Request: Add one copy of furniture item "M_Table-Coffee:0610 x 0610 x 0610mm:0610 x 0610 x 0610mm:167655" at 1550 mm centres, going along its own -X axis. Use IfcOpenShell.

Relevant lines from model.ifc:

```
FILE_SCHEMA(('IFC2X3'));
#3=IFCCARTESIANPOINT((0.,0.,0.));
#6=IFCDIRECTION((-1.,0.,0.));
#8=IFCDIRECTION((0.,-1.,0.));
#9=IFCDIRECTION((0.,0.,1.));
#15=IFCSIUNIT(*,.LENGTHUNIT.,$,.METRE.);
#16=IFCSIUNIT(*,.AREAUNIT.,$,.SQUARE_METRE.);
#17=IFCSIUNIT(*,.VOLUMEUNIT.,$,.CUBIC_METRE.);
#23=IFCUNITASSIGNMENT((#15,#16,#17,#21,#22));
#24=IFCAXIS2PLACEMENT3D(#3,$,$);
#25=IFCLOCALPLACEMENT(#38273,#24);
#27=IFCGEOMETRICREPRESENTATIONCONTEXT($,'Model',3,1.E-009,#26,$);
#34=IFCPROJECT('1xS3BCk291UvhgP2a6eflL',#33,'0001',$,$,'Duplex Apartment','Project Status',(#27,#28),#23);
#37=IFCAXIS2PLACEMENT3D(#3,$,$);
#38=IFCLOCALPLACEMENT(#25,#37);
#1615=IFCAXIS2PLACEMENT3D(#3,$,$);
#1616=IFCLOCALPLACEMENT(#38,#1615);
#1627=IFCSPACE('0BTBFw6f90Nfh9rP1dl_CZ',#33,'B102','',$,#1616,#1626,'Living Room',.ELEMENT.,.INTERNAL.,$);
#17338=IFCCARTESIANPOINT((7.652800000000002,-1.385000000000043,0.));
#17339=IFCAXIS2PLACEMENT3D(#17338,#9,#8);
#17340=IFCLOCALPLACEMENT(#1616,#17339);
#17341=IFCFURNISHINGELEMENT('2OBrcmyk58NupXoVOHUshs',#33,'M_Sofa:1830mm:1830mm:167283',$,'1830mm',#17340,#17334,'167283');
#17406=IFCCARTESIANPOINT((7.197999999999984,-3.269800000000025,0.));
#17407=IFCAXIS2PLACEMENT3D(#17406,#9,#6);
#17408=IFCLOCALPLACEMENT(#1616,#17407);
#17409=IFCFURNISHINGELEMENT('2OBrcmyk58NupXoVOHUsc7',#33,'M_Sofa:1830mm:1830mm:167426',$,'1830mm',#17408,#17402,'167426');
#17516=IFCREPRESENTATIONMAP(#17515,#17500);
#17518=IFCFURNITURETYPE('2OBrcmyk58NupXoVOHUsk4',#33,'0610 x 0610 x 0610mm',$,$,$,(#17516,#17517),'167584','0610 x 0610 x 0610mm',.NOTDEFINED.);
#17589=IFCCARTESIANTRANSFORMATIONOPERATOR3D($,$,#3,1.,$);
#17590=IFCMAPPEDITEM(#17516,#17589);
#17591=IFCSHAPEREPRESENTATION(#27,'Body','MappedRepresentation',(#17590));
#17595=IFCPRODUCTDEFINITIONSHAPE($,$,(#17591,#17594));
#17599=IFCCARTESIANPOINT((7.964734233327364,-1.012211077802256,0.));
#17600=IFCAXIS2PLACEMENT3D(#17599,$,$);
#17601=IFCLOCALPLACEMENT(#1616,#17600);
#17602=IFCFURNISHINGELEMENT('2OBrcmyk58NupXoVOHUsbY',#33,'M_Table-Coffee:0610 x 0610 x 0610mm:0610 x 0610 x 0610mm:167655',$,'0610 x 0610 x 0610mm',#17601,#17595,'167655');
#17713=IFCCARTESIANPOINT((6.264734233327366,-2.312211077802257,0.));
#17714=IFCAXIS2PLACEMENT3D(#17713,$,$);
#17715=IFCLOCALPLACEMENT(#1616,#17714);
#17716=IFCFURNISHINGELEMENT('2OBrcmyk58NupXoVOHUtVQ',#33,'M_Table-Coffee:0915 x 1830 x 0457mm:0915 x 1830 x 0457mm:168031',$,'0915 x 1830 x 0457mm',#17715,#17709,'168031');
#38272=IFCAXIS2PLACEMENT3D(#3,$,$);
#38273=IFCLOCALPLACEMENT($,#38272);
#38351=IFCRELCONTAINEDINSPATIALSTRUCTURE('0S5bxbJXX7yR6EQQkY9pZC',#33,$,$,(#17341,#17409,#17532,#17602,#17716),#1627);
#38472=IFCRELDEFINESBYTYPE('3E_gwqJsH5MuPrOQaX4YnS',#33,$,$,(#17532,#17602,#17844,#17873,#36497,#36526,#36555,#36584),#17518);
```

```python
import ifcopenshell
import ifcopenshell.api.geometry
import ifcopenshell.api.root
import ifcopenshell.util.element
import ifcopenshell.util.placement
import ifcopenshell.util.unit

model = ifcopenshell.open("model.ifc")
unit_scale = ifcopenshell.util.unit.calculate_unit_scale(model)


def reuse_history(source, copy):
    """copy_class also copies each property set's owner history, people and application; keep the originals."""
    for rel in copy.IsDefinedBy:
        if rel.is_a("IfcRelDefinesByProperties") and (history := rel.RelatingPropertyDefinition.OwnerHistory):
            rel.RelatingPropertyDefinition.OwnerHistory = source.OwnerHistory
            ifcopenshell.util.element.remove_deep2(model, history)


source = model.by_id(17602)
base = ifcopenshell.util.placement.get_local_placement(source.ObjectPlacement)
step = -base[:3, 0] * 1.55 / unit_scale

for i in range(1, 2):
    copy = ifcopenshell.api.root.copy_class(model, product=source)
    copy.Representation = ifcopenshell.util.element.copy_deep(
        model, source.Representation, exclude=["IfcGeometricRepresentationContext", "IfcRepresentationMap"]
    )
    copy.Name = "M_Table-Coffee:0610 x 0610 x 0610mm:0610 x 0610 x 0610mm"
    copy.Tag = None
    reuse_history(source, copy)
    matrix = base.copy()
    matrix[:3, 3] += i * step
    print("added at", matrix[:3, 3].round(3) + 0.0)
    ifcopenshell.api.geometry.edit_object_placement(model, product=copy, matrix=matrix, is_si=False)

model.write("model_updated.ifc")
```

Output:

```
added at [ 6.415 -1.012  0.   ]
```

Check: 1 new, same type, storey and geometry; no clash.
